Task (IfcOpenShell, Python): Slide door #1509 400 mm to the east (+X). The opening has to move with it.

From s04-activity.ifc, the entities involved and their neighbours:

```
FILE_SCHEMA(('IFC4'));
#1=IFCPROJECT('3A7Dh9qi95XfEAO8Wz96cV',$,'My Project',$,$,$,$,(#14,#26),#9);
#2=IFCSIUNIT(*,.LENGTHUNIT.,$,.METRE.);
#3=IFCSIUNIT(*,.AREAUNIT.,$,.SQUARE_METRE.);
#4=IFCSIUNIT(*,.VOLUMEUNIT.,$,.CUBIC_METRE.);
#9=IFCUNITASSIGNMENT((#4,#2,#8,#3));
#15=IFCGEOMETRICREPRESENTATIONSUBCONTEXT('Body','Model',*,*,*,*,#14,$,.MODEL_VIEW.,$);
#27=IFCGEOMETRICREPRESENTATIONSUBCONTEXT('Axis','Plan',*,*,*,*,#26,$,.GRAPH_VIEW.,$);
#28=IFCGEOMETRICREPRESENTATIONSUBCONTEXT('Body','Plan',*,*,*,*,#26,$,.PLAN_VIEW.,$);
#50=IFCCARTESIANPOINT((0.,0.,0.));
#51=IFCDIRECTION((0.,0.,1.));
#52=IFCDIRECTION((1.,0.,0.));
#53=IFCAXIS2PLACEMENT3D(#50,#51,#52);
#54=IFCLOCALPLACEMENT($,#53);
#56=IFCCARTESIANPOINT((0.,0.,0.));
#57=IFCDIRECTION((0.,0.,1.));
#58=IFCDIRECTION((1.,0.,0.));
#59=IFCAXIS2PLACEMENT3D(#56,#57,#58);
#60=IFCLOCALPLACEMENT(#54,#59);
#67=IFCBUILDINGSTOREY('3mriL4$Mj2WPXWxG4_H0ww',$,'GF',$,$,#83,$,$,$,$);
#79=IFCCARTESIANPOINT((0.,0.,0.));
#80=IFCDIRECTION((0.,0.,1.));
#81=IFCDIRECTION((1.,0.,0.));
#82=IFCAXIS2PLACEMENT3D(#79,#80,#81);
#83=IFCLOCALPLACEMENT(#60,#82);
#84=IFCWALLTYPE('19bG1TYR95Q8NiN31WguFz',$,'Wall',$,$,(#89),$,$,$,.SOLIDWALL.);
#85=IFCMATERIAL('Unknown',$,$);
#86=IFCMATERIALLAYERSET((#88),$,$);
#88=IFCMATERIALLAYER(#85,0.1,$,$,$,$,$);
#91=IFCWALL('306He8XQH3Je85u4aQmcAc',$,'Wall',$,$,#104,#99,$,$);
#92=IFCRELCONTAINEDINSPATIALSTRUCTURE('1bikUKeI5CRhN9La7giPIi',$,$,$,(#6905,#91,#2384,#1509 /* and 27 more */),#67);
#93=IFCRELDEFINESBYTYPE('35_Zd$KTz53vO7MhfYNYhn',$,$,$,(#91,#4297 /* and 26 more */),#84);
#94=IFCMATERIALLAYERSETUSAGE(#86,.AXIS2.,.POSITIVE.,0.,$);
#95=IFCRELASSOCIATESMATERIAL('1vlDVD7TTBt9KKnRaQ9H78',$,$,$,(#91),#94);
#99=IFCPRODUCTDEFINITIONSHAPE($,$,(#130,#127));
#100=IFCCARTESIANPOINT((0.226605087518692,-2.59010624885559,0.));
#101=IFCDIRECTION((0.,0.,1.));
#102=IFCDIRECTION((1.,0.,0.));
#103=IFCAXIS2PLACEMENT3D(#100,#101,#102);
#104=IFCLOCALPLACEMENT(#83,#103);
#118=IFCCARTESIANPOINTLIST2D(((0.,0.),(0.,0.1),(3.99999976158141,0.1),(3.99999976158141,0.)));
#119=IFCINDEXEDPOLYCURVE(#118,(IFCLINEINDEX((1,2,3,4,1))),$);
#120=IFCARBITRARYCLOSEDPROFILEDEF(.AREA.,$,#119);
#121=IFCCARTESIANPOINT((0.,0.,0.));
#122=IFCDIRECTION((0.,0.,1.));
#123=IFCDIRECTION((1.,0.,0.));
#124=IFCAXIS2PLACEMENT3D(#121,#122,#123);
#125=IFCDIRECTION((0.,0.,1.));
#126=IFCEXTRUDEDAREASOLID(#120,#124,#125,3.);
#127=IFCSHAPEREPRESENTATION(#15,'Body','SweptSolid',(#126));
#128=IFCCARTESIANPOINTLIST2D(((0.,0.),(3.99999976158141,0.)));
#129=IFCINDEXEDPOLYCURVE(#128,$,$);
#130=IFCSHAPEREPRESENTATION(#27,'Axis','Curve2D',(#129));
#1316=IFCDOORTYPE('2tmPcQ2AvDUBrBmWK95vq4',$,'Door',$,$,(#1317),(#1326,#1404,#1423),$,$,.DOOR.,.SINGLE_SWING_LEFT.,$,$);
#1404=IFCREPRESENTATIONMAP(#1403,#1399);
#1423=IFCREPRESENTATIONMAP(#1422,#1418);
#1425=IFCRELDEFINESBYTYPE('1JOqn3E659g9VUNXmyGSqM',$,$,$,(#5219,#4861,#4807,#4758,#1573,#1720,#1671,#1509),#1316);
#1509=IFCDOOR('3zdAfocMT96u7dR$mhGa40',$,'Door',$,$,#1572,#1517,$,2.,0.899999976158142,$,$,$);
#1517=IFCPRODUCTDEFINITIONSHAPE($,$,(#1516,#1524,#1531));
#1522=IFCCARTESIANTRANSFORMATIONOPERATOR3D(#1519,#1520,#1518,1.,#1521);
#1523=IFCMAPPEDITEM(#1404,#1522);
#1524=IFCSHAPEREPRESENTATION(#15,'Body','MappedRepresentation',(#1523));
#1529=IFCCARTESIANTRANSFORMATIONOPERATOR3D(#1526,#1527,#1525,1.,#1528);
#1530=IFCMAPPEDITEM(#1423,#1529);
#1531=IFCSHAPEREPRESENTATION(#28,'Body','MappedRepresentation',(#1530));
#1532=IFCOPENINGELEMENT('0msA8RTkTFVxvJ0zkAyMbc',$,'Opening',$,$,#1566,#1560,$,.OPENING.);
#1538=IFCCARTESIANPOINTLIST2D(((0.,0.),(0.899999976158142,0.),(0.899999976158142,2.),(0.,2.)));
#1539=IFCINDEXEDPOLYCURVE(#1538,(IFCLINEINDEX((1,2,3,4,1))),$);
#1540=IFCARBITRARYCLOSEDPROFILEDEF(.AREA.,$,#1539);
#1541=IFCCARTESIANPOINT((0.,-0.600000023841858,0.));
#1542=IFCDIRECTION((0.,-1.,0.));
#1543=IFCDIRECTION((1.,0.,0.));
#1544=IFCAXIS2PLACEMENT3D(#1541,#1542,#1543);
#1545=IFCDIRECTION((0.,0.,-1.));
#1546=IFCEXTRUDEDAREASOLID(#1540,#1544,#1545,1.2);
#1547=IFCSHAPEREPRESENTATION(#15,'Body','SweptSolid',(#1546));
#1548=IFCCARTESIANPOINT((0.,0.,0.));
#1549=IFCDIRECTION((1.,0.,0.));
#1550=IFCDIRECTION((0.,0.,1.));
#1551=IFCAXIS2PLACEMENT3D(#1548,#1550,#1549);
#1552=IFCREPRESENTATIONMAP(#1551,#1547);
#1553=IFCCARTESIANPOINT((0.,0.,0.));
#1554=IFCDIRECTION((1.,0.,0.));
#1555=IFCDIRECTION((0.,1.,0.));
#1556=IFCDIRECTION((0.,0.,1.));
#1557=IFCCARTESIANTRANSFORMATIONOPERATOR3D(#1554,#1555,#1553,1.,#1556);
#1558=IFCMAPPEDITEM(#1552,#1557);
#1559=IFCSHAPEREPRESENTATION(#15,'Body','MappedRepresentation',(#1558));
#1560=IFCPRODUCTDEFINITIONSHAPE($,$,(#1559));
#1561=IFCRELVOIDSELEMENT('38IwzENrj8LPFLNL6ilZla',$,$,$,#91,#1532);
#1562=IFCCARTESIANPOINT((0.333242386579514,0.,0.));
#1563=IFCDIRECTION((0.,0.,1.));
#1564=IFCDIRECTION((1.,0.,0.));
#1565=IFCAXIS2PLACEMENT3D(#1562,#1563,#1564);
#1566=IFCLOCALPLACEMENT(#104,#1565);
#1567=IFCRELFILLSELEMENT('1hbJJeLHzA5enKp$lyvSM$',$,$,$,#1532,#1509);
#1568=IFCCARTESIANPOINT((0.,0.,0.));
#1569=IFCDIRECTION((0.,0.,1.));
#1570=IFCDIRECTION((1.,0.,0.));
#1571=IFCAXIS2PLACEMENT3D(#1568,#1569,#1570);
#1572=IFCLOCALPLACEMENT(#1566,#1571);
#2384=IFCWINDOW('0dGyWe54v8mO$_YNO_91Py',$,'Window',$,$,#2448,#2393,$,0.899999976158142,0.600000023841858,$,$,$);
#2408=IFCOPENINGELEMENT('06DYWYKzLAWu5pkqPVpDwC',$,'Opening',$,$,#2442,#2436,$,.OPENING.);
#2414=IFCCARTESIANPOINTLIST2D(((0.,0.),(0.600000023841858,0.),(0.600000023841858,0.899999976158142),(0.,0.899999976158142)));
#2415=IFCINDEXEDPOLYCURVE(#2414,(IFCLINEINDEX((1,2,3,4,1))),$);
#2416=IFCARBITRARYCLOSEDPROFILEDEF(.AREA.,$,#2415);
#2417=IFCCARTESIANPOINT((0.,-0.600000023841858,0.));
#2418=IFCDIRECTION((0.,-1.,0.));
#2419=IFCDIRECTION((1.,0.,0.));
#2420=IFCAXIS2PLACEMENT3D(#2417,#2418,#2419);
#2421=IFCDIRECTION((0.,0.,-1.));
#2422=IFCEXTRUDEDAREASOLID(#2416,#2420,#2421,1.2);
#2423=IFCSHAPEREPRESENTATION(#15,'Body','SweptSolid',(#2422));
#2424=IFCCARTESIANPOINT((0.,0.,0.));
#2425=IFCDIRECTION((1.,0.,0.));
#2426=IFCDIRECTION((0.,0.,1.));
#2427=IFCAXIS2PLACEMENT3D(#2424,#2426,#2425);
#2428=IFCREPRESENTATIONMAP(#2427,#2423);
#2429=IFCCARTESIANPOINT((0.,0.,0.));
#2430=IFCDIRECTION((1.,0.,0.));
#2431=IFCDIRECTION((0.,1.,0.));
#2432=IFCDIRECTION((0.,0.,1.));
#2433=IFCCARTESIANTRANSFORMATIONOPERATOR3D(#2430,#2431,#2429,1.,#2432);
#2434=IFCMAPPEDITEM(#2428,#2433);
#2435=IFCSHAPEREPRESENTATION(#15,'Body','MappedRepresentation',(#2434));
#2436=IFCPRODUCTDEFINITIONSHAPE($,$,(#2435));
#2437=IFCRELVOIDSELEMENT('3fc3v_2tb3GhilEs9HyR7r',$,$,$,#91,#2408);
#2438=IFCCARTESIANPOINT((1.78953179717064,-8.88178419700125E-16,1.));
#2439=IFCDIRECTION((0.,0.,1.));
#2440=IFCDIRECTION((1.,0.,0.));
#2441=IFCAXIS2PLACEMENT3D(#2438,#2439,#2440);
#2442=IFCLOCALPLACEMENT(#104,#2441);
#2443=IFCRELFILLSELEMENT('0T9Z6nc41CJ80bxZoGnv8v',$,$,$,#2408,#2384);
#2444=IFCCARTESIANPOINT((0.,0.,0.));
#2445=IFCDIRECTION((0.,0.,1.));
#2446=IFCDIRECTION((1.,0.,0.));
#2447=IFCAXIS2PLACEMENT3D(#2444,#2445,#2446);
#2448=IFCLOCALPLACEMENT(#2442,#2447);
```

```python
import ifcopenshell
import ifcopenshell.api.geometry
import ifcopenshell.util.placement
import ifcopenshell.util.unit

model = ifcopenshell.open("s04-activity.ifc")
unit_scale = ifcopenshell.util.unit.calculate_unit_scale(model)

door = model.by_guid("3zdAfocMT96u7dR$mhGa40")
opening = door.FillsVoids[0].RelatingOpeningElement
wall = opening.VoidsElements[0].RelatingBuildingElement

wall_matrix = ifcopenshell.util.placement.get_local_placement(wall.ObjectPlacement)
shift = wall_matrix[:3, 0] * 0.4 / unit_scale
before = ifcopenshell.util.placement.get_local_placement(door.ObjectPlacement)[:3, 3].copy()

# The door is placed relative to its opening, so it follows when the opening moves.
matrix = ifcopenshell.util.placement.get_local_placement(opening.ObjectPlacement)
matrix[:3, 3] += shift
ifcopenshell.api.geometry.edit_object_placement(
    model, product=opening, matrix=matrix, is_si=False, should_transform_children=True
)

after = ifcopenshell.util.placement.get_local_placement(door.ObjectPlacement)[:3, 3]
print("door moved by", (after - before).round(3) + 0.0)

model.write("s04-activity_edited.ifc")
```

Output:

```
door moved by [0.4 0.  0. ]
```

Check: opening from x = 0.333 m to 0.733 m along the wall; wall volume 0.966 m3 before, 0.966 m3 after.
